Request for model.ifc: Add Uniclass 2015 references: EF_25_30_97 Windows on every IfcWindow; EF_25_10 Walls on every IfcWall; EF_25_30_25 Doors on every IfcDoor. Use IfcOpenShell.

First a look at what the model holds.

```python
import ifcopenshell

model = ifcopenshell.open("model.ifc")
print(model.schema)
print("classifications:", [c.Name for c in model.by_type("IfcClassification")])
for ifc_class in ("IfcDoor", "IfcRoof", "IfcStair", "IfcWall", "IfcWindow"):
    print(ifc_class, len(model.by_type(ifc_class)))
```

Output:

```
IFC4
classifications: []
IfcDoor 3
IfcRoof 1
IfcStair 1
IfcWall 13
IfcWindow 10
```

```python
import ifcopenshell
import ifcopenshell.api.classification

model = ifcopenshell.open("model.ifc")

system = ifcopenshell.api.classification.add_classification(model, classification="Uniclass 2015")

codes = {
    "IfcWindow": ("EF_25_30_97", "Windows"),
    "IfcWall": ("EF_25_10", "Walls"),
    "IfcDoor": ("EF_25_30_25", "Doors"),
}
for ifc_class, (code, name) in codes.items():
    products = model.by_type(ifc_class)
    ifcopenshell.api.classification.add_reference(
        model, products=products, classification=system, identification=code, name=name
    )
    print(code, len(products))

model.write("model_v2.ifc")
```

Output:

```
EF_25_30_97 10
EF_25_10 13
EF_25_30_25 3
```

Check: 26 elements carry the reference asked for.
